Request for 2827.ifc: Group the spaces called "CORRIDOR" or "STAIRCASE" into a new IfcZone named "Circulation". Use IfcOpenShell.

First a look at what the model holds.

```python
import ifcopenshell

model = ifcopenshell.open("2827.ifc")
print(model.schema)
seen = {}
for space in model.by_type("IfcSpace"):
    seen[space.LongName] = seen.get(space.LongName, 0) + 1
for name, count in sorted(seen.items(), key=str):
    print(count, "x", name)
print("zones:", [z.Name for z in model.by_type("IfcZone")][:20])
```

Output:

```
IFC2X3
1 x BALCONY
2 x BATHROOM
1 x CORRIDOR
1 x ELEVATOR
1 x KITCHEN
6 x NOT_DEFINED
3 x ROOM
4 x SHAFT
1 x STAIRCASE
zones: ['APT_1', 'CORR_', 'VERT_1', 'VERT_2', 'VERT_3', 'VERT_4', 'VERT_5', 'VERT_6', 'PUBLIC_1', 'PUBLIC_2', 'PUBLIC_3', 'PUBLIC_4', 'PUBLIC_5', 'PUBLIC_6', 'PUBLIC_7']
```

```python
import ifcopenshell
import ifcopenshell.api.group
import ifcopenshell.api.root

model = ifcopenshell.open("2827.ifc")

names = {"CORRIDOR", "STAIRCASE"}
spaces = [s for s in model.by_type("IfcSpace") if s.LongName in names]

zone = ifcopenshell.api.root.create_entity(model, ifc_class="IfcZone", name="Circulation")
ifcopenshell.api.group.assign_group(model, products=spaces, group=zone)
print(len(spaces), "spaces in", zone.Name)

model.write("2827_updated.ifc")
```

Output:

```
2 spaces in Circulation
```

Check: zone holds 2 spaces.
